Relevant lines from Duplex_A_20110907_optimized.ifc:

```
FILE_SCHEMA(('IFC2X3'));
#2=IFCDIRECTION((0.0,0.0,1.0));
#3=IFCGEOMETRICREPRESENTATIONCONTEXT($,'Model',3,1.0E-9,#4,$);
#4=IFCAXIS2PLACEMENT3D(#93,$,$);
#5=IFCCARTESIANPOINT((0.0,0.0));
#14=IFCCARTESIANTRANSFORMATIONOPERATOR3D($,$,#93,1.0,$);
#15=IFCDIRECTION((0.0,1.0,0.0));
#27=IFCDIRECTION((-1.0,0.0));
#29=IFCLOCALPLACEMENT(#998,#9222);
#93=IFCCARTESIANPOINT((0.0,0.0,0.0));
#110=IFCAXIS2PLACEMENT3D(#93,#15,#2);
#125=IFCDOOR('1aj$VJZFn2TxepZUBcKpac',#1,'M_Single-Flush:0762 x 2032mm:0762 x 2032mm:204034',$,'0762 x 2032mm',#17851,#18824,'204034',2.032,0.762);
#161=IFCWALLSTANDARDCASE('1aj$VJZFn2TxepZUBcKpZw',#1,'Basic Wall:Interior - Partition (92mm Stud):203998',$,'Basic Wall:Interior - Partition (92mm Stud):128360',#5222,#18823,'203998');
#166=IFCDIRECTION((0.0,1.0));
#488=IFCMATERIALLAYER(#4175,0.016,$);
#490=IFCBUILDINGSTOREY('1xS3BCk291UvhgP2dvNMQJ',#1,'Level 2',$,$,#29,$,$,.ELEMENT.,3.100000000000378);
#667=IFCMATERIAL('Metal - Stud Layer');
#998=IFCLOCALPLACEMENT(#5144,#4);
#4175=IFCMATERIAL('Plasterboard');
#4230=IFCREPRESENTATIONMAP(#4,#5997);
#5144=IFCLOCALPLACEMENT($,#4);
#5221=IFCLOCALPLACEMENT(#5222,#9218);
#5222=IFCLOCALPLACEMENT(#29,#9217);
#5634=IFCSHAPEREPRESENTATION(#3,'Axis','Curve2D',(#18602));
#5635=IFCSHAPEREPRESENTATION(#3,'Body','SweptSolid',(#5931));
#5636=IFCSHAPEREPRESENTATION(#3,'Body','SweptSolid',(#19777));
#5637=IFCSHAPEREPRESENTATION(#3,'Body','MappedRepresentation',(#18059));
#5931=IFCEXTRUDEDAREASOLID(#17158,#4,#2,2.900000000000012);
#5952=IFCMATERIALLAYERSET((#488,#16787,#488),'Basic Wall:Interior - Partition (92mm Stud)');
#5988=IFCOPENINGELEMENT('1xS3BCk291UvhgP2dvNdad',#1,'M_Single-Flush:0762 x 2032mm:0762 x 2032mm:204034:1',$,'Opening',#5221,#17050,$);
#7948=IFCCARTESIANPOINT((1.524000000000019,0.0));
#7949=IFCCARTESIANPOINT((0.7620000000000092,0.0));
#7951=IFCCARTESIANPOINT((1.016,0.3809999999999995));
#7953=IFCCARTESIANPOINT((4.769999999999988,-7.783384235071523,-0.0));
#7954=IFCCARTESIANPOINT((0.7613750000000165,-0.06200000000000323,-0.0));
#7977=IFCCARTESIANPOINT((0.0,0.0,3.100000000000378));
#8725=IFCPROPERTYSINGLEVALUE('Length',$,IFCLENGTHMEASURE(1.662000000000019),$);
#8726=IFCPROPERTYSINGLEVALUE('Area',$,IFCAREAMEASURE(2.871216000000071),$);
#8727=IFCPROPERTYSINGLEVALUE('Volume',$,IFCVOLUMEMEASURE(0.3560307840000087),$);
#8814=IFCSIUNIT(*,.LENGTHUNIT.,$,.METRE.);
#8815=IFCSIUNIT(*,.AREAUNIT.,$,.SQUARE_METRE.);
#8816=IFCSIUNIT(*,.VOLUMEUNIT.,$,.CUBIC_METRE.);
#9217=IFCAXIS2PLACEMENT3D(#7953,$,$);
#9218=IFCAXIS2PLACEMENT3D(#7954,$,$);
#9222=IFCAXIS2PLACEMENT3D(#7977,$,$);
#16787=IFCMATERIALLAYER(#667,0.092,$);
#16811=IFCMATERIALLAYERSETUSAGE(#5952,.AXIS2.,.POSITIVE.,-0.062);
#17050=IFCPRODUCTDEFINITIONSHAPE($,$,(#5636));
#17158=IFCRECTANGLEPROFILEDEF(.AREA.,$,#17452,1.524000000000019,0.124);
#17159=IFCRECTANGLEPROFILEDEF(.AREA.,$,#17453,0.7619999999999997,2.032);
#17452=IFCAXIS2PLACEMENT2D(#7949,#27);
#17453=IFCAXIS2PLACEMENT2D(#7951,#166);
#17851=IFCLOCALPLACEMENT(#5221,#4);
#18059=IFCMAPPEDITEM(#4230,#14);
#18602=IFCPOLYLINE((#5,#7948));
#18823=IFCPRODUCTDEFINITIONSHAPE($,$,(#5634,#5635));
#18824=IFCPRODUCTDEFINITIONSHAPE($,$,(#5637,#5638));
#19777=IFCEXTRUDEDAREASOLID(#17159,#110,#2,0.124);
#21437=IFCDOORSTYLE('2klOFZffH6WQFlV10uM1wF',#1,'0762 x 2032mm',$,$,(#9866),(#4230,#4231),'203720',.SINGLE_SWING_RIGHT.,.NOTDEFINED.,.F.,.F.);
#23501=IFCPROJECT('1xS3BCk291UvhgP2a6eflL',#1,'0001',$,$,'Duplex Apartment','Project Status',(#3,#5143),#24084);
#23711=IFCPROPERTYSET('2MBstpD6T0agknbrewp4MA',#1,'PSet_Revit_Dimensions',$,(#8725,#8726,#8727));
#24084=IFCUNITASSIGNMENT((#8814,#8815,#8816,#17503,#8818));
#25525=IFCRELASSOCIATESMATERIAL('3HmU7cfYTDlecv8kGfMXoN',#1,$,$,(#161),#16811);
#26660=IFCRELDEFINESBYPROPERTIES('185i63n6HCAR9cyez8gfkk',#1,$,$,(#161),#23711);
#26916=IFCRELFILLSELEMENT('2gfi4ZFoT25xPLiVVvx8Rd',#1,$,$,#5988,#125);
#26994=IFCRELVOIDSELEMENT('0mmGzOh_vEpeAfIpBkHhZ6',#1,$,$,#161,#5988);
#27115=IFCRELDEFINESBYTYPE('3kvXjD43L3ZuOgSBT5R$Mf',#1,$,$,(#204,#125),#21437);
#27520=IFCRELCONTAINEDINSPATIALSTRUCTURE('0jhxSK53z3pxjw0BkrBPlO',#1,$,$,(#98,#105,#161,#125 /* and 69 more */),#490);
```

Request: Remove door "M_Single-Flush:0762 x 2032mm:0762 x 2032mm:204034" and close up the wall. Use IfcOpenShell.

```python
import ifcopenshell
import ifcopenshell.api.feature
import ifcopenshell.api.pset
import ifcopenshell.api.root
import ifcopenshell.geom
import ifcopenshell.util.element
import ifcopenshell.util.shape
import ifcopenshell.util.unit

model = ifcopenshell.open("Duplex_A_20110907_optimized.ifc")
area_scale = ifcopenshell.util.unit.calculate_unit_scale(model, "AREAUNIT")
volume_scale = ifcopenshell.util.unit.calculate_unit_scale(model, "VOLUMEUNIT")
settings = ifcopenshell.geom.settings()


def volume(element):
    """Net volume in cubic metres, openings subtracted."""
    shape = ifcopenshell.geom.create_shape(settings, element)
    return ifcopenshell.util.shape.get_volume(shape.geometry)


door = model.by_id(125)
opening = door.FillsVoids[0].RelatingOpeningElement
wall = opening.VoidsElements[0].RelatingBuildingElement
before = volume(wall)

ifcopenshell.api.root.remove_product(model, product=door)
ifcopenshell.api.feature.remove_feature(model, feature=opening)

after = volume(wall)
thickness = 0.124  # wall thickness in metres

# Update the wall's stored quantities.
pset = model.by_id(ifcopenshell.util.element.get_pset(wall, "PSet_Revit_Dimensions", should_inherit=False)["id"])
ifcopenshell.api.pset.edit_pset(model, pset=pset, properties={
    "Area": model.create_entity("IfcAreaMeasure", after / thickness / area_scale),
    "Volume": model.create_entity("IfcVolumeMeasure", after / volume_scale),
})

print(f"wall volume {before:.3f} -> {after:.3f} m3")

model.write("Duplex_A_20110907_optimized_edited.ifc")
```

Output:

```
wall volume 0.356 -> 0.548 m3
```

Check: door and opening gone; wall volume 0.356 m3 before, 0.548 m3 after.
